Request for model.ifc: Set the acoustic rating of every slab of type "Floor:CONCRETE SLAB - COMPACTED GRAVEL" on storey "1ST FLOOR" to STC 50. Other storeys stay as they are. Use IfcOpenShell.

First a look at what the model holds.

```python
import ifcopenshell
import ifcopenshell.util.element

model = ifcopenshell.open("model.ifc")
print(model.schema)
storey = next(s for s in model.by_type("IfcBuildingStorey") if s.Name == "1ST FLOOR")
slabs = [e for e in ifcopenshell.util.element.get_decomposition(storey) if e.is_a("IfcSlab")]
seen = {}
for e in slabs:
    element_type = ifcopenshell.util.element.get_type(e)
    key = (element_type.Name if element_type != e and element_type else None, ifcopenshell.util.element.get_pset(e, "Pset_SlabCommon", "AcousticRating"))
    seen[key] = seen.get(key, 0) + 1
for (name, value), count in sorted(seen.items(), key=str):
    print(count, "x", name, "|", value)
```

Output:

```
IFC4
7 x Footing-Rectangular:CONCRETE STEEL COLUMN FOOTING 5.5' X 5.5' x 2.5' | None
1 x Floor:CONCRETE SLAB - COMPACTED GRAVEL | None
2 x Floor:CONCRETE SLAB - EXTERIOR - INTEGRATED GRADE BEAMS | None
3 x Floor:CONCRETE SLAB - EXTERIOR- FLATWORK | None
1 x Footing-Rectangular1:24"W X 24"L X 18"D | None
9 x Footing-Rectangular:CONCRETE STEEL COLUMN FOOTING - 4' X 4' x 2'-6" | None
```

```python
import ifcopenshell
import ifcopenshell.api.pset
import ifcopenshell.util.element

model = ifcopenshell.open("model.ifc")

storey = next(s for s in model.by_type("IfcBuildingStorey") if s.Name == "1ST FLOOR")
slabs = [e for e in ifcopenshell.util.element.get_decomposition(storey) if e.is_a("IfcSlab")]

count = 0
for e in slabs:
    element_type = ifcopenshell.util.element.get_type(e)
    if element_type in (None, e) or element_type.Name != "Floor:CONCRETE SLAB - COMPACTED GRAVEL":
        continue
    # add_pset returns the element's existing set when there is one.
    pset = ifcopenshell.api.pset.add_pset(model, product=e, name="Pset_SlabCommon")
    ifcopenshell.api.pset.edit_pset(model, pset=pset, properties={"AcousticRating": "STC 50"})
    count += 1

print(count, "slabs updated")

model.write("model_updated.ifc")
```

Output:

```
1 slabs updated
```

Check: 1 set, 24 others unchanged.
